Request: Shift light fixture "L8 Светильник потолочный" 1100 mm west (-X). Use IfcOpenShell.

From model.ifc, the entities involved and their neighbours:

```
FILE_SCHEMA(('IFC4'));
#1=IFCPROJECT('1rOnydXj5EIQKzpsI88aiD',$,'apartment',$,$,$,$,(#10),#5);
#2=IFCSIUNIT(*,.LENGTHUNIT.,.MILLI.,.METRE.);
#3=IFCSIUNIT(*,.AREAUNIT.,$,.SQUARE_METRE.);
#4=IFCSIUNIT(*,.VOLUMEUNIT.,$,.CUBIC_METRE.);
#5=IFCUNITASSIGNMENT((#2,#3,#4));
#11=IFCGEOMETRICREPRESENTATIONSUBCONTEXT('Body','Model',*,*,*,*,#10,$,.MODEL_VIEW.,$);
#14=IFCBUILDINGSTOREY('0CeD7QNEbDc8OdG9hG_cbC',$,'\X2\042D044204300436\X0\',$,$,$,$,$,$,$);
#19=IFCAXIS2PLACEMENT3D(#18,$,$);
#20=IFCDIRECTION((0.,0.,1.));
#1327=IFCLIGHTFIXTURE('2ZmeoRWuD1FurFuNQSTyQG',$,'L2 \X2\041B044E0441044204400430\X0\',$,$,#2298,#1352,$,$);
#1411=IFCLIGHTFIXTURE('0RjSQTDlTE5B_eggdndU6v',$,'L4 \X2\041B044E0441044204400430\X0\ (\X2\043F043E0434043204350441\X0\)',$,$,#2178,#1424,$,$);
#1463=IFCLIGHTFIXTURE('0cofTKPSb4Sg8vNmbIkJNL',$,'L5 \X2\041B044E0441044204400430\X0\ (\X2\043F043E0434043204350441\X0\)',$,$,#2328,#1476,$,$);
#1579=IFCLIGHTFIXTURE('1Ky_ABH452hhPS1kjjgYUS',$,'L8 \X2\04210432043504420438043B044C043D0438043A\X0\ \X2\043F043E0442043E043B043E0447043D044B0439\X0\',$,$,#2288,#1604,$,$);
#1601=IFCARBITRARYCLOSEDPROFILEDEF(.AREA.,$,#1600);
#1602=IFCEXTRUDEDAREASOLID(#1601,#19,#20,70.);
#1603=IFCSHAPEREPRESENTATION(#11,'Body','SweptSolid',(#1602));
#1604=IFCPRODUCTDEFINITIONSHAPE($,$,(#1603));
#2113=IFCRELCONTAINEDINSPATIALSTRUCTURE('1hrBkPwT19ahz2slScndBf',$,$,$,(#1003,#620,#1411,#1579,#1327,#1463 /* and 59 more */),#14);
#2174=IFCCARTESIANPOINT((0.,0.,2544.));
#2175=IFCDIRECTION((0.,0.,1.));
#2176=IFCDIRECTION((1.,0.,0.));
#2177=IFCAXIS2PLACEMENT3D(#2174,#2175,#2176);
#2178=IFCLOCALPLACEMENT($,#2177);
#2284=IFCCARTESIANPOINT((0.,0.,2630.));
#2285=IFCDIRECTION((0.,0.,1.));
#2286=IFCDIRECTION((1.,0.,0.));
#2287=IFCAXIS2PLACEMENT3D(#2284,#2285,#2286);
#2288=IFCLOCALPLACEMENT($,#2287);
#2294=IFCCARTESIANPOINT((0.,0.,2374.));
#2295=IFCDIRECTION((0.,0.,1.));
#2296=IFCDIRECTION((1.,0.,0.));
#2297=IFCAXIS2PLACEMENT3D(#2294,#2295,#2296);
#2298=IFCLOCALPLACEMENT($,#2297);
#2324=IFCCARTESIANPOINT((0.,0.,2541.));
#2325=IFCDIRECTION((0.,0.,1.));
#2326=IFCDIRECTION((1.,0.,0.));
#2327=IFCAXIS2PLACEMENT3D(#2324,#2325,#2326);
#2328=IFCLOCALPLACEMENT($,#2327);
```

```python
import ifcopenshell
import ifcopenshell.api.geometry
import ifcopenshell.util.placement
import ifcopenshell.util.unit

model = ifcopenshell.open("model.ifc")
unit_scale = ifcopenshell.util.unit.calculate_unit_scale(model)

item = model.by_guid("1Ky_ABH452hhPS1kjjgYUS")
matrix = ifcopenshell.util.placement.get_local_placement(item.ObjectPlacement)
matrix[0, 3] -= 1.1 / unit_scale
ifcopenshell.api.geometry.edit_object_placement(model, product=item, matrix=matrix, is_si=False)

print(ifcopenshell.util.placement.get_local_placement(item.ObjectPlacement).round(3) + 0.0)

model.write("model_edited.ifc")
```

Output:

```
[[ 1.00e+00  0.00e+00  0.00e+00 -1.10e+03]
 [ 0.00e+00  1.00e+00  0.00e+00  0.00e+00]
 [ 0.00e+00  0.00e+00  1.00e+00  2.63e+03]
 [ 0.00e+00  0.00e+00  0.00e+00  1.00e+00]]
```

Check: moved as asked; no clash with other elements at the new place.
